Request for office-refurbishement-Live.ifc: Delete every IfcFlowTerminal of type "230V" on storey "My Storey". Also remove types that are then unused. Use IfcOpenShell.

First a look at what the model holds.

```python
import ifcopenshell
import ifcopenshell.util.element

model = ifcopenshell.open("office-refurbishement-Live.ifc")
print(model.schema)
storey = next(s for s in model.by_type("IfcBuildingStorey") if s.Name == "My Storey")
terminals = [e for e in ifcopenshell.util.element.get_decomposition(storey) if e.is_a("IfcFlowTerminal")]
seen = {}
for e in terminals:
    element_type = ifcopenshell.util.element.get_type(e)
    name = element_type.Name if element_type not in (None, e) else None
    seen[name] = seen.get(name, 0) + 1
for name, count in sorted(seen.items(), key=str):
    print(count, "x", name)
```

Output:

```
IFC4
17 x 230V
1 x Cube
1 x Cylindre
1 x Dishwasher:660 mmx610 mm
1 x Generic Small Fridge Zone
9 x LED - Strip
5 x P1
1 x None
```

```python
import ifcopenshell
import ifcopenshell.api.root
import ifcopenshell.util.element

model = ifcopenshell.open("office-refurbishement-Live.ifc")

storey = next(s for s in model.by_type("IfcBuildingStorey") if s.Name == "My Storey")
terminals = [e for e in ifcopenshell.util.element.get_decomposition(storey) if e.is_a("IfcFlowTerminal")]
targets = [e for e in terminals if (t := ifcopenshell.util.element.get_type(e)) not in (None, e) and t.Name == "230V"]
types = {ifcopenshell.util.element.get_type(e) for e in targets} - {None, *targets}

for e in targets:
    ifcopenshell.api.root.remove_product(model, product=e)
print(len(targets), "removed")

unused = [t for t in types if not ifcopenshell.util.element.get_types(t)]
for t in unused:
    ifcopenshell.api.root.remove_product(model, product=t)
print(len(unused), "unused types removed")

model.write("office-refurbishement-Live_v2.ifc")
```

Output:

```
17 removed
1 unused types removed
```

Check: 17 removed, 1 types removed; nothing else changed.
